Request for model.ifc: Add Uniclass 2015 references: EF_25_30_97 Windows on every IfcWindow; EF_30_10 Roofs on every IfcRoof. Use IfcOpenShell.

First a look at what the model holds.

```python
import ifcopenshell

model = ifcopenshell.open("model.ifc")
print(model.schema)
print("classifications:", [c.Name for c in model.by_type("IfcClassification")])
for ifc_class in ("IfcDoor", "IfcRoof", "IfcStair", "IfcWall", "IfcWindow"):
    print(ifc_class, len(model.by_type(ifc_class)))
```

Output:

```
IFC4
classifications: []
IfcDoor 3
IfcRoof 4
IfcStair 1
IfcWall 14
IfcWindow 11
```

```python
import ifcopenshell
import ifcopenshell.api.classification

model = ifcopenshell.open("model.ifc")

system = ifcopenshell.api.classification.add_classification(model, classification="Uniclass 2015")

codes = {
    "IfcWindow": ("EF_25_30_97", "Windows"),
    "IfcRoof": ("EF_30_10", "Roofs"),
}
for ifc_class, (code, name) in codes.items():
    products = model.by_type(ifc_class)
    ifcopenshell.api.classification.add_reference(
        model, products=products, classification=system, identification=code, name=name
    )
    print(code, len(products))

model.write("model_v2.ifc")
```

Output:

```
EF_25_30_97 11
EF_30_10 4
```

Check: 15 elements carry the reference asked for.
